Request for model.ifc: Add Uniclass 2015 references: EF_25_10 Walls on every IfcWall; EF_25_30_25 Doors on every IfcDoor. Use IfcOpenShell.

First a look at what the model holds.

```python
import ifcopenshell

model = ifcopenshell.open("model.ifc")
print(model.schema)
print("classifications:", [c.Name for c in model.by_type("IfcClassification")])
for ifc_class in ("IfcDoor", "IfcRoof", "IfcStair", "IfcWall", "IfcWindow"):
    print(ifc_class, len(model.by_type(ifc_class)))
```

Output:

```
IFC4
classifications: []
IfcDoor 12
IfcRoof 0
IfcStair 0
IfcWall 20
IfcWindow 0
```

```python
import ifcopenshell
import ifcopenshell.api.classification

model = ifcopenshell.open("model.ifc")

system = ifcopenshell.api.classification.add_classification(model, classification="Uniclass 2015")

codes = {
    "IfcWall": ("EF_25_10", "Walls"),
    "IfcDoor": ("EF_25_30_25", "Doors"),
}
for ifc_class, (code, name) in codes.items():
    products = model.by_type(ifc_class)
    ifcopenshell.api.classification.add_reference(
        model, products=products, classification=system, identification=code, name=name
    )
    print(code, len(products))

model.write("model_updated.ifc")
```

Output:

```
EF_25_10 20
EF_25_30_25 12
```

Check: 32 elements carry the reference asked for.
